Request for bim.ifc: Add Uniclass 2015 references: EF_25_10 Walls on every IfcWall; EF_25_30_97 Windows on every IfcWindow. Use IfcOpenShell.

First a look at what the model holds.

```python
import ifcopenshell

model = ifcopenshell.open("bim.ifc")
print(model.schema)
print("classifications:", [c.Name for c in model.by_type("IfcClassification")])
for ifc_class in ("IfcDoor", "IfcRoof", "IfcStair", "IfcWall", "IfcWindow"):
    print(ifc_class, len(model.by_type(ifc_class)))
```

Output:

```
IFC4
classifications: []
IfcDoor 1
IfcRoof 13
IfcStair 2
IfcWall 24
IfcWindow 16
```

```python
import ifcopenshell
import ifcopenshell.api.classification

model = ifcopenshell.open("bim.ifc")

system = ifcopenshell.api.classification.add_classification(model, classification="Uniclass 2015")

codes = {
    "IfcWall": ("EF_25_10", "Walls"),
    "IfcWindow": ("EF_25_30_97", "Windows"),
}
for ifc_class, (code, name) in codes.items():
    products = model.by_type(ifc_class)
    ifcopenshell.api.classification.add_reference(
        model, products=products, classification=system, identification=code, name=name
    )
    print(code, len(products))

model.write("bim_edited.ifc")
```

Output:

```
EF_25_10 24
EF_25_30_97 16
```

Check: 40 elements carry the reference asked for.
